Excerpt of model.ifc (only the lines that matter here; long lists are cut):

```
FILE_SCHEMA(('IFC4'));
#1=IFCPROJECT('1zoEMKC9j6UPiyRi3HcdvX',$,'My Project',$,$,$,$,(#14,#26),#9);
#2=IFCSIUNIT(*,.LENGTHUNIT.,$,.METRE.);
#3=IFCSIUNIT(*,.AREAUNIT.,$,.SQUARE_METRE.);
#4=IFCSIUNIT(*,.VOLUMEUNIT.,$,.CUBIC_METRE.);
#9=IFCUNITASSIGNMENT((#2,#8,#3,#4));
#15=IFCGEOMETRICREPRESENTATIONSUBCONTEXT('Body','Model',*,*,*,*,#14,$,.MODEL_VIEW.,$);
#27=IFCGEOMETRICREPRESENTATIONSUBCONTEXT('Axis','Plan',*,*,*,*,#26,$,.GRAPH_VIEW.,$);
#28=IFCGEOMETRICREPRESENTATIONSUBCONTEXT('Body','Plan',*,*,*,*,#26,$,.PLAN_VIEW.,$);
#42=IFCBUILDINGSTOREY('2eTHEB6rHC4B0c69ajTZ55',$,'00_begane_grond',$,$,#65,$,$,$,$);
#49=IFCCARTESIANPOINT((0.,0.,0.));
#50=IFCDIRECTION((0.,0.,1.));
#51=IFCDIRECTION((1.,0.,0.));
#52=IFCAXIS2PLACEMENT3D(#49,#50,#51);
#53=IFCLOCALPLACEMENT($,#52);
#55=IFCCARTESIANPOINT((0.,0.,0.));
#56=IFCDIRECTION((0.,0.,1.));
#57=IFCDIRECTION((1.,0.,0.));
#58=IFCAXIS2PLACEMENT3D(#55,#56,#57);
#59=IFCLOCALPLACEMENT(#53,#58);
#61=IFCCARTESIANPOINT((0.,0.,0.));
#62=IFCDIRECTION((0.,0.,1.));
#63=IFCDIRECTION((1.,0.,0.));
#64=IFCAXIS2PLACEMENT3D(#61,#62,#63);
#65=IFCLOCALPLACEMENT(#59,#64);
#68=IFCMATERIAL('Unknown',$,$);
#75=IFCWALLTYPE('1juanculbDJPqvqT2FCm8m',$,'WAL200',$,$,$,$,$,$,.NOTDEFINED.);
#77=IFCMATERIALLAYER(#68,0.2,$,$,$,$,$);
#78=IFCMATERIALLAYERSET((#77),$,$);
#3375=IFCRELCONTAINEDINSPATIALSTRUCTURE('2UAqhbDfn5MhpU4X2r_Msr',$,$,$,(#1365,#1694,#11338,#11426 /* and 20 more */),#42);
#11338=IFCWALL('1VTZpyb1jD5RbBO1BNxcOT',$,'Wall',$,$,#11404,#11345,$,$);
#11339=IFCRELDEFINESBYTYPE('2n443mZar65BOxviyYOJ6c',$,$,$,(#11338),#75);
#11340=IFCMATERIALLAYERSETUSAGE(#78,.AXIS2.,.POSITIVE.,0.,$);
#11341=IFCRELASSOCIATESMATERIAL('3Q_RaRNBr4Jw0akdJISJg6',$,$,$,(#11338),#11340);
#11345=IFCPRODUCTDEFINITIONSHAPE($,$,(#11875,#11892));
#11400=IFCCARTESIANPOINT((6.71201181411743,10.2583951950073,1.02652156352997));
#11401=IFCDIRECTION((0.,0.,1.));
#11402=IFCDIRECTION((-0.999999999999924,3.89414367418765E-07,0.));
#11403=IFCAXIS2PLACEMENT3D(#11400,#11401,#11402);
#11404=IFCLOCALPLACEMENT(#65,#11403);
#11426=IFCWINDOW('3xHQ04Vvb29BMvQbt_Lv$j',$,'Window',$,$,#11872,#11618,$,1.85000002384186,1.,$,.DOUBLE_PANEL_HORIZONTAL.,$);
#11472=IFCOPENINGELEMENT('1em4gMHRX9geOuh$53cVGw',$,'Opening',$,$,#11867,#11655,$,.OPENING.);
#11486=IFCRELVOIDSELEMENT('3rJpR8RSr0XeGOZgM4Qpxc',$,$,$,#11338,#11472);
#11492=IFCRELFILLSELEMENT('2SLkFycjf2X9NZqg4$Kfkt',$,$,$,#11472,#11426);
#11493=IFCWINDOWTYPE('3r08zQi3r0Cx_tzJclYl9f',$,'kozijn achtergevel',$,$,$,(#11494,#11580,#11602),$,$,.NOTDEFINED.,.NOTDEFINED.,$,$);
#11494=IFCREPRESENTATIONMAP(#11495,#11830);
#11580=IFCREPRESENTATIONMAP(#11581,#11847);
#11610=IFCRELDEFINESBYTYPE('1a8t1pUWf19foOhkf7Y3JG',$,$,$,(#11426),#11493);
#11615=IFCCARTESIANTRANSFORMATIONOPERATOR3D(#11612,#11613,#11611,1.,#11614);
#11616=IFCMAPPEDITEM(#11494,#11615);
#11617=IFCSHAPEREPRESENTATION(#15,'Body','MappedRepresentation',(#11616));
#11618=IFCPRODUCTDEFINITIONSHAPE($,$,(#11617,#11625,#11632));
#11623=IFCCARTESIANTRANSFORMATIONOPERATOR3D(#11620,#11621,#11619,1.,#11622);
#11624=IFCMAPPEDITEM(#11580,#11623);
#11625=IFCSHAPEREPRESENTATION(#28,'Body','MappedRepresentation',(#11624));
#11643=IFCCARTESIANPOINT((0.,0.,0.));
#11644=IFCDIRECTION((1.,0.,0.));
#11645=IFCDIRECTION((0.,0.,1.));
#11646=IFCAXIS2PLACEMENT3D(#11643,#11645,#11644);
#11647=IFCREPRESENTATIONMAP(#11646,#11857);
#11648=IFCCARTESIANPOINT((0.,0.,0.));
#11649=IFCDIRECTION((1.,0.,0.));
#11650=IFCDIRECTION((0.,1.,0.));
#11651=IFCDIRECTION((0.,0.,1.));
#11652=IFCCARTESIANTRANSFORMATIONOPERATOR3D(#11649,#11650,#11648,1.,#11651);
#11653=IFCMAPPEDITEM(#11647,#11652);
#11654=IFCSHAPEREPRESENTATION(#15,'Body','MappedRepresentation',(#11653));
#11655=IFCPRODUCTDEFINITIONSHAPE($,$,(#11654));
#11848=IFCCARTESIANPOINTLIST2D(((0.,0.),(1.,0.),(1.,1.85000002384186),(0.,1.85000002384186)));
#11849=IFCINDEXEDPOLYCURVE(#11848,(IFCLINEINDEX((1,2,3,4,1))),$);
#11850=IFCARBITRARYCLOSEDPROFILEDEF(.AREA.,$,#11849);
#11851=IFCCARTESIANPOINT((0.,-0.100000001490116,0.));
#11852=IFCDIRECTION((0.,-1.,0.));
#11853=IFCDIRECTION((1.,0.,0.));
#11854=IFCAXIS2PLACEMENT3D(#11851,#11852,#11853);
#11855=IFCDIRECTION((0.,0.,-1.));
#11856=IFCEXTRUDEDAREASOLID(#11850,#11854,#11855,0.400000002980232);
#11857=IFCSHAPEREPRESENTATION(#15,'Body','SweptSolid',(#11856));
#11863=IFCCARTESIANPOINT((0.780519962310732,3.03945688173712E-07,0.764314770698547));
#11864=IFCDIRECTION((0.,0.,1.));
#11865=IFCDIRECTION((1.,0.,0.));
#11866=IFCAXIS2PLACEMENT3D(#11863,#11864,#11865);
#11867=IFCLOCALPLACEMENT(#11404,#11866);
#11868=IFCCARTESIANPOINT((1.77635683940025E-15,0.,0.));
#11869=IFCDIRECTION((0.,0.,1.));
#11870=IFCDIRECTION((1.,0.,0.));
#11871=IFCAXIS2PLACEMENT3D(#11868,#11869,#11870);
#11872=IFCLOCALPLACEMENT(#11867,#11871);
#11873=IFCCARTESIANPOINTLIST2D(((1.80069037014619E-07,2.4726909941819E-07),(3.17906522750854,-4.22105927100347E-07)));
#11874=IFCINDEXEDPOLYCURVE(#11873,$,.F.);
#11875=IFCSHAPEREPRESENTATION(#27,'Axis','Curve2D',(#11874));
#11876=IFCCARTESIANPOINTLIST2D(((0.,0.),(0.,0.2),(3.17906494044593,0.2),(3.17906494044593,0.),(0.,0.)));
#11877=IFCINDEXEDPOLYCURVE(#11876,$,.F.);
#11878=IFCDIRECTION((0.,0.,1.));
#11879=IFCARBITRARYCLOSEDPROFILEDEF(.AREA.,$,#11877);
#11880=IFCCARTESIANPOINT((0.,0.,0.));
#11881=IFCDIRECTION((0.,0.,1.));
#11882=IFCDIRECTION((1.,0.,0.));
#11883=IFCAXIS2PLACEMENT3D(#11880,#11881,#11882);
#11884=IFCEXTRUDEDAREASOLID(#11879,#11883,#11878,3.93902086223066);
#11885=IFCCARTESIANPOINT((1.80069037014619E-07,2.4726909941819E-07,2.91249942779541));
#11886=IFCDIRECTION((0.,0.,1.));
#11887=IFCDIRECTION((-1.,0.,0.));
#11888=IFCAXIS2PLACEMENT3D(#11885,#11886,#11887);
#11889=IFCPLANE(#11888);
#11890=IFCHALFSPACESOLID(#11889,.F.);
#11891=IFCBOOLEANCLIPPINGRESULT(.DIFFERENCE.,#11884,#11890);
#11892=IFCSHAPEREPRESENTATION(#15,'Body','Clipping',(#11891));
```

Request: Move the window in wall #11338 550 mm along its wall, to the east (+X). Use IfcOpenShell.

```python
import ifcopenshell
import ifcopenshell.api.geometry
import ifcopenshell.util.placement
import ifcopenshell.util.unit

model = ifcopenshell.open("model.ifc")
unit_scale = ifcopenshell.util.unit.calculate_unit_scale(model)

window = model.by_guid("3xHQ04Vvb29BMvQbt_Lv$j")
opening = window.FillsVoids[0].RelatingOpeningElement
wall = opening.VoidsElements[0].RelatingBuildingElement

wall_matrix = ifcopenshell.util.placement.get_local_placement(wall.ObjectPlacement)
shift = wall_matrix[:3, 0] * -0.55 / unit_scale
before = ifcopenshell.util.placement.get_local_placement(window.ObjectPlacement)[:3, 3].copy()

# The window is placed relative to its opening, so it follows when the opening moves.
matrix = ifcopenshell.util.placement.get_local_placement(opening.ObjectPlacement)
matrix[:3, 3] += shift
ifcopenshell.api.geometry.edit_object_placement(
    model, product=opening, matrix=matrix, is_si=False, should_transform_children=True
)

after = ifcopenshell.util.placement.get_local_placement(window.ObjectPlacement)[:3, 3]
print("window moved by", (after - before).round(3) + 0.0)

model.write("model_rev.ifc")
```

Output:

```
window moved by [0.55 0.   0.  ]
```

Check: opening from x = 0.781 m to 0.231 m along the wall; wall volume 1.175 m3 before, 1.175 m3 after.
